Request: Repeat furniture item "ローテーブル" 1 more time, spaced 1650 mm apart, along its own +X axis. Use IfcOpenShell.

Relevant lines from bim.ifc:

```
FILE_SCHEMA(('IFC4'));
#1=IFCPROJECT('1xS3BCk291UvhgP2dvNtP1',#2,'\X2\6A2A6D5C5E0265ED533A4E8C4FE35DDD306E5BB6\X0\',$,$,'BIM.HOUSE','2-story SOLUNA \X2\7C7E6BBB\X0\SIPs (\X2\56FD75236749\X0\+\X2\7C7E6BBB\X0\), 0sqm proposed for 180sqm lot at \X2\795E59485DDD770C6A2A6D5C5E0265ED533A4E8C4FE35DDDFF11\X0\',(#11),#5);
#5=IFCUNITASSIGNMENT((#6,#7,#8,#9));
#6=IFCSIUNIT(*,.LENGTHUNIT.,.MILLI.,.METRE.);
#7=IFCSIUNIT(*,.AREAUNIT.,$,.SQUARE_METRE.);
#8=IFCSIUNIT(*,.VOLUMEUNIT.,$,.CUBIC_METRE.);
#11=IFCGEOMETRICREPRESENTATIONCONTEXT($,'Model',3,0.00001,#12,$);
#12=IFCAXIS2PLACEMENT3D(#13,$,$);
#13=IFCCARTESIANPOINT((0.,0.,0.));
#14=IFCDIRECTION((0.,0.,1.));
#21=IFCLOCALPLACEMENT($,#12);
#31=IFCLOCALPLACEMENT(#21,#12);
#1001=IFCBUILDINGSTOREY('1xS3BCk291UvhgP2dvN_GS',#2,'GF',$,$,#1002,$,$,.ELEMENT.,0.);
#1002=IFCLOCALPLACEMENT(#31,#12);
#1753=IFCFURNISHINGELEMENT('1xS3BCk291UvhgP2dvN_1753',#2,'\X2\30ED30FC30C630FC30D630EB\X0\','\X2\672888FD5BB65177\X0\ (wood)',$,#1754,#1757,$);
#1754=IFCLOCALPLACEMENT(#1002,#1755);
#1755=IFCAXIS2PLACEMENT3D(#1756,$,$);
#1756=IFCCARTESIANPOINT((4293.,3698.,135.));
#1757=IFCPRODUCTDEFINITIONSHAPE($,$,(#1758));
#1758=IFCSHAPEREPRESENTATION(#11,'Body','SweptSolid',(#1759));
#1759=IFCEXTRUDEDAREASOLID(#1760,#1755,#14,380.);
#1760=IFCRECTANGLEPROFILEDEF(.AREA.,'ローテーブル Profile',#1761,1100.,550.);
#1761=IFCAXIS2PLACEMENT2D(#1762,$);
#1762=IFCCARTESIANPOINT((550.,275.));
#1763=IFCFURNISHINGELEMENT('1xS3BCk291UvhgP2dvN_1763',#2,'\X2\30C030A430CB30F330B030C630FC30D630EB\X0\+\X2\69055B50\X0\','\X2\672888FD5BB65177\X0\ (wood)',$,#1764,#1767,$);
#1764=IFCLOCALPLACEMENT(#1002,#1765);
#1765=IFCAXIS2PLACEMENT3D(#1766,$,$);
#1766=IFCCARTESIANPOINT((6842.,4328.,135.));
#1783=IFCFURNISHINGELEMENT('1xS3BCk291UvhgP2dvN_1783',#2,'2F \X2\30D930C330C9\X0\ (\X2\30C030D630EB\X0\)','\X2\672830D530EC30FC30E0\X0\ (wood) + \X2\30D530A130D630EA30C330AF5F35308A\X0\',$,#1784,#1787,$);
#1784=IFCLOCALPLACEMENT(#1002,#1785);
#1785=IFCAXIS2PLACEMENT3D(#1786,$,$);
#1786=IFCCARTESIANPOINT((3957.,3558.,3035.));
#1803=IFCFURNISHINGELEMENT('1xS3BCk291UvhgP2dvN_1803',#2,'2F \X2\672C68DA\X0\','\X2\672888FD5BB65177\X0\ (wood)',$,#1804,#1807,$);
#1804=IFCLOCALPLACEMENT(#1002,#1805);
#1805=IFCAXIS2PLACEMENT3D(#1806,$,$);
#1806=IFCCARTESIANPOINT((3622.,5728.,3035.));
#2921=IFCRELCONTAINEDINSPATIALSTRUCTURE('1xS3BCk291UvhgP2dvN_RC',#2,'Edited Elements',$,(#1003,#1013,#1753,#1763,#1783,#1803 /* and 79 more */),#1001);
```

```python
import ifcopenshell
import ifcopenshell.api.geometry
import ifcopenshell.api.root
import ifcopenshell.util.element
import ifcopenshell.util.placement
import ifcopenshell.util.unit

model = ifcopenshell.open("bim.ifc")
unit_scale = ifcopenshell.util.unit.calculate_unit_scale(model)


def reuse_history(source, copy):
    """copy_class also copies each property set's owner history, people and application; keep the originals."""
    for rel in copy.IsDefinedBy:
        if rel.is_a("IfcRelDefinesByProperties") and (history := rel.RelatingPropertyDefinition.OwnerHistory):
            rel.RelatingPropertyDefinition.OwnerHistory = source.OwnerHistory
            ifcopenshell.util.element.remove_deep2(model, history)


source = model.by_guid("1xS3BCk291UvhgP2dvN_1753")
base = ifcopenshell.util.placement.get_local_placement(source.ObjectPlacement)
step = base[:3, 0] * 1.65 / unit_scale

for i in range(1, 2):
    copy = ifcopenshell.api.root.copy_class(model, product=source)
    copy.Representation = ifcopenshell.util.element.copy_deep(
        model, source.Representation, exclude=["IfcGeometricRepresentationContext", "IfcRepresentationMap"]
    )
    reuse_history(source, copy)
    matrix = base.copy()
    matrix[:3, 3] += i * step
    print("added at", matrix[:3, 3].round(3) + 0.0)
    ifcopenshell.api.geometry.edit_object_placement(model, product=copy, matrix=matrix, is_si=False)

model.write("bim_edited.ifc")
```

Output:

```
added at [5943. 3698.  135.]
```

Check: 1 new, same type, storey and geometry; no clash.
